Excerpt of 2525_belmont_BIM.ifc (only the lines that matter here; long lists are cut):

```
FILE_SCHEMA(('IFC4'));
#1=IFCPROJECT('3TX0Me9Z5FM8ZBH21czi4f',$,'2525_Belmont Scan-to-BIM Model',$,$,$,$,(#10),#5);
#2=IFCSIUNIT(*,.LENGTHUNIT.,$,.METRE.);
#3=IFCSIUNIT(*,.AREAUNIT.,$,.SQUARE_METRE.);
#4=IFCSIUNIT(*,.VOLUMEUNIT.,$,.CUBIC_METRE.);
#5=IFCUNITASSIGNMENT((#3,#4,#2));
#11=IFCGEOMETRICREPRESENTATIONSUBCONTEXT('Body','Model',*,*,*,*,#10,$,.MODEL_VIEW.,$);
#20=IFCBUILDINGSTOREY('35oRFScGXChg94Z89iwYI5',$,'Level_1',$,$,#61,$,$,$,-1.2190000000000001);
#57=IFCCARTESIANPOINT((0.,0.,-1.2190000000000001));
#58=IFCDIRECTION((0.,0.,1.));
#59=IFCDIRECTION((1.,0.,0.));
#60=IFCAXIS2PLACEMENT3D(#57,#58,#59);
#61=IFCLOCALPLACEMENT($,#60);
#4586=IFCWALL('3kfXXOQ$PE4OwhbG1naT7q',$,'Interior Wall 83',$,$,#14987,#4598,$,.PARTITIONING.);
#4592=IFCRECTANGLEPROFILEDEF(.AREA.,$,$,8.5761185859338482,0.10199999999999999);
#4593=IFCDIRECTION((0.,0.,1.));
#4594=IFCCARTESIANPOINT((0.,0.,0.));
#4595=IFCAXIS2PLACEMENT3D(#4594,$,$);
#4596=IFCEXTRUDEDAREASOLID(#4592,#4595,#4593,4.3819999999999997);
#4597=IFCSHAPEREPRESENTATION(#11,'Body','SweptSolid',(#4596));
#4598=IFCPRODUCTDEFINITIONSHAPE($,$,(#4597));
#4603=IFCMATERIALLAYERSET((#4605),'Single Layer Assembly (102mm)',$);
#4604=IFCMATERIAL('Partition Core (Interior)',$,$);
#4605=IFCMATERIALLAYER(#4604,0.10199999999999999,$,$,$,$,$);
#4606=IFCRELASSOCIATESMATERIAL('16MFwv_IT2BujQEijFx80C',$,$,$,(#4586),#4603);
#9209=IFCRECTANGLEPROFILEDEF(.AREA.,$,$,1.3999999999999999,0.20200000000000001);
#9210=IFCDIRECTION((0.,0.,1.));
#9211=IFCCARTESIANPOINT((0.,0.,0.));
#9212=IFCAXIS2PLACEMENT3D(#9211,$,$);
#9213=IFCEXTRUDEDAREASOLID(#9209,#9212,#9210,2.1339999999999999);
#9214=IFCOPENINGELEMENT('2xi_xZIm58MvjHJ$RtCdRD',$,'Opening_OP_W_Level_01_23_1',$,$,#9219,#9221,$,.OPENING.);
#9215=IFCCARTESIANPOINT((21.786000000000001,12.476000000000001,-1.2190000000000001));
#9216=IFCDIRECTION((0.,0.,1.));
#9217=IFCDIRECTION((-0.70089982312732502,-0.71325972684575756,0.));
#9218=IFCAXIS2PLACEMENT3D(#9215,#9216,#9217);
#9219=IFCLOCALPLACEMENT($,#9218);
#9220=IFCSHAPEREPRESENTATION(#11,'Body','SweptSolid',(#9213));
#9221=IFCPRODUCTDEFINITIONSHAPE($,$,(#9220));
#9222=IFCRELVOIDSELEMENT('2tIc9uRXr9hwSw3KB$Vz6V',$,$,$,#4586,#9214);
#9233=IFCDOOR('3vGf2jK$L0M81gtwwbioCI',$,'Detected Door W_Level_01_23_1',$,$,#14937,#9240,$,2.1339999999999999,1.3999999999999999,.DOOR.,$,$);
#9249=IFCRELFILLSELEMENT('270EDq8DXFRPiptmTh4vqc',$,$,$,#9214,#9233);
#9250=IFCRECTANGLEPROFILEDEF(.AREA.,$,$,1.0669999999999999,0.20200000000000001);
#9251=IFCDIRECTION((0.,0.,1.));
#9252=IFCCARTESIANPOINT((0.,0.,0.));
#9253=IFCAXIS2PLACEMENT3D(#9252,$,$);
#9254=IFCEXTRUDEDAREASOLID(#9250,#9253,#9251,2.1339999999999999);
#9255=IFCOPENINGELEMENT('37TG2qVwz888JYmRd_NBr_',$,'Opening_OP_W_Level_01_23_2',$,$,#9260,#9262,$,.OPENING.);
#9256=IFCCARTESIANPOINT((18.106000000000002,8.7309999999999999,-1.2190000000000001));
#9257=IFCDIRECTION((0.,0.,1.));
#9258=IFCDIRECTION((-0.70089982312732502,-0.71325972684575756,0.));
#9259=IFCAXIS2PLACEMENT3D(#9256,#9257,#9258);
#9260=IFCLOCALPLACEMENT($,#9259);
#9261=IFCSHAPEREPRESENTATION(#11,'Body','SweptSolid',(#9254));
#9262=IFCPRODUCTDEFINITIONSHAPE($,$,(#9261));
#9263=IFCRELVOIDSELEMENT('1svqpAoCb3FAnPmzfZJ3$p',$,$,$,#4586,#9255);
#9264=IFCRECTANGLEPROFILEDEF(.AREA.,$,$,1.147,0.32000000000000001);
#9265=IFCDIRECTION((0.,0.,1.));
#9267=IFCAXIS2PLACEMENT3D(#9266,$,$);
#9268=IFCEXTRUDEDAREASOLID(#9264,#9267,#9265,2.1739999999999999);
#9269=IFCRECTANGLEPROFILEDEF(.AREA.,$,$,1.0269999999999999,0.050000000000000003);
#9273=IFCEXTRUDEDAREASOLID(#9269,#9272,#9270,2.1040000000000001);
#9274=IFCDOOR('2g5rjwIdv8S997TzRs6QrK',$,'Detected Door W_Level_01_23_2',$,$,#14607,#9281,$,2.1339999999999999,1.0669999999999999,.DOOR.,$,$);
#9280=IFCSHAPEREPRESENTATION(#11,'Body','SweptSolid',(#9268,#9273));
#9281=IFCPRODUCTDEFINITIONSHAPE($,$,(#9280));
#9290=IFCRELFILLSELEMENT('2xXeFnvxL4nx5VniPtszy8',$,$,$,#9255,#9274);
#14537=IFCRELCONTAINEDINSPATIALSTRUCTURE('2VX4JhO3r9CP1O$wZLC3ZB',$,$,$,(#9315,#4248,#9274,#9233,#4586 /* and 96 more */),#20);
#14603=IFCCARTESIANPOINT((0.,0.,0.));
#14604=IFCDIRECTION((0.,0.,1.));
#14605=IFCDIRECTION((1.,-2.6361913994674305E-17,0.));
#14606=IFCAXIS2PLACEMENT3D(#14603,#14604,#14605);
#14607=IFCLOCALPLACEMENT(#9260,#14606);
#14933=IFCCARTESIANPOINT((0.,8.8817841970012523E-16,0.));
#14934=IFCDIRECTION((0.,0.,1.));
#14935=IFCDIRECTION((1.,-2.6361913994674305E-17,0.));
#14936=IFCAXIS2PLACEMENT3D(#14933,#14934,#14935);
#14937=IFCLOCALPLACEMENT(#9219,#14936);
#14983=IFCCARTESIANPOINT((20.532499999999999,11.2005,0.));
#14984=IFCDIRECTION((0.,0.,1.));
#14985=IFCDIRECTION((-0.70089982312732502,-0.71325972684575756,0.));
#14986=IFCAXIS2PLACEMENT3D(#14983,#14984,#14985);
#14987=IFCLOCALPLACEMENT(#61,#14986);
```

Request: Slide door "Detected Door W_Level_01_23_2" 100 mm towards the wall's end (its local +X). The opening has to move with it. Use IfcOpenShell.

```python
import ifcopenshell
import ifcopenshell.api.geometry
import ifcopenshell.util.placement

model = ifcopenshell.open("2525_belmont_BIM.ifc")

door = model.by_guid("2g5rjwIdv8S997TzRs6QrK")
opening = door.FillsVoids[0].RelatingOpeningElement
wall = opening.VoidsElements[0].RelatingBuildingElement

wall_matrix = ifcopenshell.util.placement.get_local_placement(wall.ObjectPlacement)
shift = wall_matrix[:3, 0] * 0.1
before = ifcopenshell.util.placement.get_local_placement(door.ObjectPlacement)[:3, 3].copy()

# The door is placed relative to its opening, so it follows when the opening moves.
matrix = ifcopenshell.util.placement.get_local_placement(opening.ObjectPlacement)
matrix[:3, 3] += shift
ifcopenshell.api.geometry.edit_object_placement(
    model, product=opening, matrix=matrix, is_si=False, should_transform_children=True
)

after = ifcopenshell.util.placement.get_local_placement(door.ObjectPlacement)[:3, 3]
print("door moved by", (after - before).round(3) + 0.0)

model.write("2525_belmont_BIM_v2.ifc")
```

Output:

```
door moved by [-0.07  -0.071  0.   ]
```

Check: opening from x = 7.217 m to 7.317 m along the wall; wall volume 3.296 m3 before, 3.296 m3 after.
